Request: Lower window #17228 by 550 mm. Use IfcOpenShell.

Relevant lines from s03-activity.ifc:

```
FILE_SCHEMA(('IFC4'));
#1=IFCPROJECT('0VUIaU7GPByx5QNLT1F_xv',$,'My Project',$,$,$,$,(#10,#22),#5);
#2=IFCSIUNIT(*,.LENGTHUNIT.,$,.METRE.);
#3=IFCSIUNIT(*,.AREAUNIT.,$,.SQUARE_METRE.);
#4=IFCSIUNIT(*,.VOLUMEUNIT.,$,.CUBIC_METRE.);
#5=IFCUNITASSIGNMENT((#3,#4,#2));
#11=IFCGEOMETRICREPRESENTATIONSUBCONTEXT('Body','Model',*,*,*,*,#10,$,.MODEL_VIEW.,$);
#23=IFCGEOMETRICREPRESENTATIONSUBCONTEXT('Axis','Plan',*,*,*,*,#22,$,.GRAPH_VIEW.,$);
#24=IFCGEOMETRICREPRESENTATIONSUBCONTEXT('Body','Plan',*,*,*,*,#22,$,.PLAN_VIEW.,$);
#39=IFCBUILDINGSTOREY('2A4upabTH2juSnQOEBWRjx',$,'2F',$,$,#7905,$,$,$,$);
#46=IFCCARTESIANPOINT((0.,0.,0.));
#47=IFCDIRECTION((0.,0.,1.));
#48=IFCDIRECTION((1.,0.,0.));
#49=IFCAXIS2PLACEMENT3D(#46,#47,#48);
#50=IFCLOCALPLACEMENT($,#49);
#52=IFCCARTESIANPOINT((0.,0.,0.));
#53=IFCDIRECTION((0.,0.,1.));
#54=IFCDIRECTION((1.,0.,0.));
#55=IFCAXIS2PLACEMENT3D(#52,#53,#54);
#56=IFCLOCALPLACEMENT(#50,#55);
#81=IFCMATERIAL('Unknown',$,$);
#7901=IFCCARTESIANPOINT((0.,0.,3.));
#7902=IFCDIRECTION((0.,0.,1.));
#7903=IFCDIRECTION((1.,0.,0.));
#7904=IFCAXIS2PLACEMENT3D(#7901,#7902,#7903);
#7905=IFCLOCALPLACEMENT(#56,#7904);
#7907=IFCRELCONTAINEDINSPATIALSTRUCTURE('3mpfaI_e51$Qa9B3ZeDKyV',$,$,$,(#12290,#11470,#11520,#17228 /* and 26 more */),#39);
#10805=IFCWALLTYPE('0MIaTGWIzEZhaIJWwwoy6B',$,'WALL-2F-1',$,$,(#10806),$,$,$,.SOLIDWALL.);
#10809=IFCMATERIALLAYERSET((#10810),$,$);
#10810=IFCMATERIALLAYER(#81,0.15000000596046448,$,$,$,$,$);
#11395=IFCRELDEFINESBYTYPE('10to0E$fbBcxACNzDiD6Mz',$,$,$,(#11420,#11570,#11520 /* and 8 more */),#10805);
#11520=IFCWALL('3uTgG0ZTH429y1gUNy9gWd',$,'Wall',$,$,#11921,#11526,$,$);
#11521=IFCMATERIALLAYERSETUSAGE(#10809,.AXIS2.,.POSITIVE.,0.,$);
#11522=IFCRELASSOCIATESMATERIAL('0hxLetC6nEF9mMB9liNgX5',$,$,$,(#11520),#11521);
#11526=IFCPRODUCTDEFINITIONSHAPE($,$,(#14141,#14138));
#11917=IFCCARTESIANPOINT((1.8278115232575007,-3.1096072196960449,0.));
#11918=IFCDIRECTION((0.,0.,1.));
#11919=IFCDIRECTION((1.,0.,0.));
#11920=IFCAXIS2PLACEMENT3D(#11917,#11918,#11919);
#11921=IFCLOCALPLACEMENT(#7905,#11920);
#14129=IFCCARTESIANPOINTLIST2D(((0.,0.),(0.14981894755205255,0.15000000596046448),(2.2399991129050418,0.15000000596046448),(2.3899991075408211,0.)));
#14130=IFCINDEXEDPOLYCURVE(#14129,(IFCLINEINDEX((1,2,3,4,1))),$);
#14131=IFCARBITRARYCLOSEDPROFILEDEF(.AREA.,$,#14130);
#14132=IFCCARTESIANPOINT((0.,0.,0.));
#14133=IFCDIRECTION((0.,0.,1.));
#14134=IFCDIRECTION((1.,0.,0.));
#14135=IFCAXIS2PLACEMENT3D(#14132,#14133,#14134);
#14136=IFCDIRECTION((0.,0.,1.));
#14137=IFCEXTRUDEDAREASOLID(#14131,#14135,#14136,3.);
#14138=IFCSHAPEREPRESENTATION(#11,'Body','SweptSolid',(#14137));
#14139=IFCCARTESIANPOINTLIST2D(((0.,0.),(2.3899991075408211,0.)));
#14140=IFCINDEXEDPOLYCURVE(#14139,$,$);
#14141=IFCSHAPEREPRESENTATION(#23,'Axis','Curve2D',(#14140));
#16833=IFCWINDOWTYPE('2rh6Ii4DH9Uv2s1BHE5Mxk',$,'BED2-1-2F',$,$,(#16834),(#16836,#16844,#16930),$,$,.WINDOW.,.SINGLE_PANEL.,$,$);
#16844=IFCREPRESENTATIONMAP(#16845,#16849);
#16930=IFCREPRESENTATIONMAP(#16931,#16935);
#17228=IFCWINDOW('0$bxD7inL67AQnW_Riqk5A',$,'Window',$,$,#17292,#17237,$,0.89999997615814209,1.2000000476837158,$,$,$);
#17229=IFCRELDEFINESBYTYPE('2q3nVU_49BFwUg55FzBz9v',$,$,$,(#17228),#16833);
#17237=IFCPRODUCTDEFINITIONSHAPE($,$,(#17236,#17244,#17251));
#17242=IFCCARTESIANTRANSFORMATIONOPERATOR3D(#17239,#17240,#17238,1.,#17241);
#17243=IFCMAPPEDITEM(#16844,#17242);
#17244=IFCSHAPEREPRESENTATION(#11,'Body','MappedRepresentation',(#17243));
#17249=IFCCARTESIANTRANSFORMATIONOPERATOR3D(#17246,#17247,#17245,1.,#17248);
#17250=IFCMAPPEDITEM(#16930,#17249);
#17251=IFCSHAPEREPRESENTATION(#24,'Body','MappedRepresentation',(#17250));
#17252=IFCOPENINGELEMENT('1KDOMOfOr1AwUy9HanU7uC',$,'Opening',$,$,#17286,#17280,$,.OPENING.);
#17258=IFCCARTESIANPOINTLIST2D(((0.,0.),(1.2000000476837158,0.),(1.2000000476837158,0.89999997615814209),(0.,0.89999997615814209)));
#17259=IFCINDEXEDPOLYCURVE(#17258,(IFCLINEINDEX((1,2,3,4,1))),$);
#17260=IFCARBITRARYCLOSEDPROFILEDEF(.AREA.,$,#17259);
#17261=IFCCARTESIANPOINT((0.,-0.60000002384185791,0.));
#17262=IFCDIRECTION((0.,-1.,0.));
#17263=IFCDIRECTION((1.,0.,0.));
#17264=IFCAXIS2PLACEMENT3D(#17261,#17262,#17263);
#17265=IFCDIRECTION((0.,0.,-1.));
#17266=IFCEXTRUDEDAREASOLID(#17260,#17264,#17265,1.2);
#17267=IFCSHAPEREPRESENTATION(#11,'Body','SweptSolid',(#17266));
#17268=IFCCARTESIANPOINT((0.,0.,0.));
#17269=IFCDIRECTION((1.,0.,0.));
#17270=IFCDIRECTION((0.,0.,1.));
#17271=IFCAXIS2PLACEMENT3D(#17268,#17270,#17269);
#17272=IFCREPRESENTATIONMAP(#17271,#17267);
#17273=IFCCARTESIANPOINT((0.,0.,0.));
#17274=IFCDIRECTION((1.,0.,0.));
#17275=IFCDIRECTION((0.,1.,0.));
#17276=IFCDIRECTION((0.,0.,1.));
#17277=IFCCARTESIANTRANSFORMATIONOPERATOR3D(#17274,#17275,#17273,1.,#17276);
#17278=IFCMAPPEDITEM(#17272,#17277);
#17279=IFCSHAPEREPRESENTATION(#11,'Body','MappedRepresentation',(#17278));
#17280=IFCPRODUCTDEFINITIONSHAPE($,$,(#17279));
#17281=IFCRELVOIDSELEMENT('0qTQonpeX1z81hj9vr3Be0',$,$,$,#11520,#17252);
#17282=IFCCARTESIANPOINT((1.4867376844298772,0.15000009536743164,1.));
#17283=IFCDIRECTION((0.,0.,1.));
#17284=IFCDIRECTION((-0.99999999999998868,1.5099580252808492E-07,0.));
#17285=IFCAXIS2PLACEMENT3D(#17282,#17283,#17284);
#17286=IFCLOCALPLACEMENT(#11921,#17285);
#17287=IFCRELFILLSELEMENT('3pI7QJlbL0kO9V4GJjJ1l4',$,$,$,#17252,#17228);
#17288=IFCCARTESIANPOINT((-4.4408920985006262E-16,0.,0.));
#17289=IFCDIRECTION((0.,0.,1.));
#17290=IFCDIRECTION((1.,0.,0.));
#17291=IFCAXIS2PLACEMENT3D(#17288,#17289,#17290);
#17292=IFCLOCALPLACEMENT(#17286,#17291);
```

```python
import numpy as np
import ifcopenshell
import ifcopenshell.api.geometry
import ifcopenshell.util.placement
import ifcopenshell.util.unit

model = ifcopenshell.open("s03-activity.ifc")
unit_scale = ifcopenshell.util.unit.calculate_unit_scale(model)

window = model.by_guid("0$bxD7inL67AQnW_Riqk5A")
opening = window.FillsVoids[0].RelatingOpeningElement
dz = -0.55 / unit_scale

shift = np.array([0.0, 0.0, dz])
# The window is placed relative to its opening, so it follows when the opening moves.
matrix = ifcopenshell.util.placement.get_local_placement(opening.ObjectPlacement)
matrix[:3, 3] += shift
ifcopenshell.api.geometry.edit_object_placement(
    model, product=opening, matrix=matrix, is_si=False, should_transform_children=True
)

print(f"moved by {dz * unit_scale:+.3f} m")

model.write("s03-activity_rev.ifc")
```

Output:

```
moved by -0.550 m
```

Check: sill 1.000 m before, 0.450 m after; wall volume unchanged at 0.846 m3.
